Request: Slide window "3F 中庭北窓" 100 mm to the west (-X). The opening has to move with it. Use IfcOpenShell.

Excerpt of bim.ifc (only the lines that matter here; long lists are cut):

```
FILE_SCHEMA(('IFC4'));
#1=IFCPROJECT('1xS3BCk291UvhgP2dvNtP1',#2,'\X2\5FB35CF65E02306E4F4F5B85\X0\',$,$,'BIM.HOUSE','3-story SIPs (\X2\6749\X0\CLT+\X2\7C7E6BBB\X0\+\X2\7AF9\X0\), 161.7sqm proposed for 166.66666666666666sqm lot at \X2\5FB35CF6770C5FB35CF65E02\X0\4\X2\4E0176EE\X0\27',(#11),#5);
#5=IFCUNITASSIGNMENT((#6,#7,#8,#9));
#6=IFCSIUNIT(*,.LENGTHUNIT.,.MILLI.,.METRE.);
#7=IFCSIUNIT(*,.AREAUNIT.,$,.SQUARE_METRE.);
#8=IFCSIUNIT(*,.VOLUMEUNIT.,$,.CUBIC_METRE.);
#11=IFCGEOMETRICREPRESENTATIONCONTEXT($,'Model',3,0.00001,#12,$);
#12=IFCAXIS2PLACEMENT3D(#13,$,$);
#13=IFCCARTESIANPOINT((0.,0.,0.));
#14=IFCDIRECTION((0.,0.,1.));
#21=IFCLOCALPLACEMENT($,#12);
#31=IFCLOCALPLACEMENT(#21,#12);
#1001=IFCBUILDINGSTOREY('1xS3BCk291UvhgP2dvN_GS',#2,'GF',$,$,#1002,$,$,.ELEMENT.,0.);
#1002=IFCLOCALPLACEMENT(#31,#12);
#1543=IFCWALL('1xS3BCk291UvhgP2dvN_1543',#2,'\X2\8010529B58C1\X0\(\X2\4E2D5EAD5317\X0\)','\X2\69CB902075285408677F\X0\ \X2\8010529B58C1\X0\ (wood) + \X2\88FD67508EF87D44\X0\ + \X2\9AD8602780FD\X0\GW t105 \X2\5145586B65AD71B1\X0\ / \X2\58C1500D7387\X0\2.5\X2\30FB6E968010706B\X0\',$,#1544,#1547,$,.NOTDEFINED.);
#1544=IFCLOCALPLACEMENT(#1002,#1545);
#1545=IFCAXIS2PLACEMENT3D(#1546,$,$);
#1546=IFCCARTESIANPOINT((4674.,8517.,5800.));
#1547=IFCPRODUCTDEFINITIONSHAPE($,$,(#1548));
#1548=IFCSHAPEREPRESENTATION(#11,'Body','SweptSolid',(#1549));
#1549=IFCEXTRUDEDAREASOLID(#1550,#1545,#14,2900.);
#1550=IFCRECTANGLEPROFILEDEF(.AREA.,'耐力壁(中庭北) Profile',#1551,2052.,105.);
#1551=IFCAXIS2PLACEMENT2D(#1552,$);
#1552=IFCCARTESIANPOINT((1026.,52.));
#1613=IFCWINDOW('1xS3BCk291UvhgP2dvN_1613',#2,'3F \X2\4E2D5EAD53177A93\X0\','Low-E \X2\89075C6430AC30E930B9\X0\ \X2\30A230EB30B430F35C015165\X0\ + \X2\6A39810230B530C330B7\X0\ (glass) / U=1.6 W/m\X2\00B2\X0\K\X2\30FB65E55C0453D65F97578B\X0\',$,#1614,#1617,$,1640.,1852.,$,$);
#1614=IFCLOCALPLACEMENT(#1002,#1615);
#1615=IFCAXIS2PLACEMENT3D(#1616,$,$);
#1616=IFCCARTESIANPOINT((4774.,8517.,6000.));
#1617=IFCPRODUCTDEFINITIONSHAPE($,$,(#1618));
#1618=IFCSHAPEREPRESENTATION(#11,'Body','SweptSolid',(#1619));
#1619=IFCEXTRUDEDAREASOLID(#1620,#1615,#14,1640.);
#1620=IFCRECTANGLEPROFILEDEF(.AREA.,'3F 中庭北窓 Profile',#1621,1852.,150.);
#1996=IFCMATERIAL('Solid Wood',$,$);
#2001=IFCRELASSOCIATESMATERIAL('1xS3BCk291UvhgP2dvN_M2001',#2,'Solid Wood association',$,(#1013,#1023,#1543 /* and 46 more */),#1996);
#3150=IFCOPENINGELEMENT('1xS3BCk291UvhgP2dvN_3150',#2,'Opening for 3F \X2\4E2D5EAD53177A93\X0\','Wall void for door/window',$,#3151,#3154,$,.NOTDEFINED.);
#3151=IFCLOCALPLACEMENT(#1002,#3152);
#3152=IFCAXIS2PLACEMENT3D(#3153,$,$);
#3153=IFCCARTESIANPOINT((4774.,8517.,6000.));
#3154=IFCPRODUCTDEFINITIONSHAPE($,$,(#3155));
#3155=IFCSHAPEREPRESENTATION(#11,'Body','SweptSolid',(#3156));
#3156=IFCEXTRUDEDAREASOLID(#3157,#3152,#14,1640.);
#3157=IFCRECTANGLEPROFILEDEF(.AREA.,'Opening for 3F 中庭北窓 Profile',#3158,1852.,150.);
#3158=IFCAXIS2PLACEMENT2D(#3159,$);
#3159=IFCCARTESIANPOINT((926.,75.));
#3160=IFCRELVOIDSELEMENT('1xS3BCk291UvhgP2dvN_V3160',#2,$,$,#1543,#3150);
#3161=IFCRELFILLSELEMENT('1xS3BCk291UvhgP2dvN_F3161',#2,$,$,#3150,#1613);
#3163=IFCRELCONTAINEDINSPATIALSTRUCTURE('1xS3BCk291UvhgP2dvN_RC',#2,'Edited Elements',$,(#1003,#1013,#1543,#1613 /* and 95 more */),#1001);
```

```python
import ifcopenshell
import ifcopenshell.api.geometry
import ifcopenshell.util.placement

model = ifcopenshell.open("bim.ifc")

window = model.by_id(1613)
opening = window.FillsVoids[0].RelatingOpeningElement
wall = opening.VoidsElements[0].RelatingBuildingElement

wall_matrix = ifcopenshell.util.placement.get_local_placement(wall.ObjectPlacement)
shift = wall_matrix[:3, 0] * -100.0
before = ifcopenshell.util.placement.get_local_placement(window.ObjectPlacement)[:3, 3].copy()

# The window is not placed relative to its opening, so move both.
for product in (opening, window):
    matrix = ifcopenshell.util.placement.get_local_placement(product.ObjectPlacement)
    matrix[:3, 3] += shift
    ifcopenshell.api.geometry.edit_object_placement(model, product=product, matrix=matrix, is_si=False)

after = ifcopenshell.util.placement.get_local_placement(window.ObjectPlacement)[:3, 3]
print("window moved by", (after - before).round(3) + 0.0)

model.write("bim_rev.ifc")
```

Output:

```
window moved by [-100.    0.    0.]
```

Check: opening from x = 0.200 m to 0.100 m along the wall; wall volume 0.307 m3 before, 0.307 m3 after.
